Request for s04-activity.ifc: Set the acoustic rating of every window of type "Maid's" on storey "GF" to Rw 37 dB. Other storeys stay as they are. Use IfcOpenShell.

First a look at what the model holds.

```python
import ifcopenshell
import ifcopenshell.util.element

model = ifcopenshell.open("s04-activity.ifc")
print(model.schema)
storey = next(s for s in model.by_type("IfcBuildingStorey") if s.Name == "GF")
windows = [e for e in ifcopenshell.util.element.get_decomposition(storey) if e.is_a("IfcWindow")]
seen = {}
for e in windows:
    element_type = ifcopenshell.util.element.get_type(e)
    key = (element_type.Name if element_type != e and element_type else None, ifcopenshell.util.element.get_pset(e, "Pset_WindowCommon", "AcousticRating"))
    seen[key] = seen.get(key, 0) + 1
for (name, value), count in sorted(seen.items(), key=str):
    print(count, "x", name, "|", value)
```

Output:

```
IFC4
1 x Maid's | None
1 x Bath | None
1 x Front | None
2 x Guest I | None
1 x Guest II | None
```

```python
import ifcopenshell
import ifcopenshell.api.pset
import ifcopenshell.util.element

model = ifcopenshell.open("s04-activity.ifc")

storey = next(s for s in model.by_type("IfcBuildingStorey") if s.Name == "GF")
windows = [e for e in ifcopenshell.util.element.get_decomposition(storey) if e.is_a("IfcWindow")]

count = 0
for e in windows:
    element_type = ifcopenshell.util.element.get_type(e)
    if element_type in (None, e) or element_type.Name != "Maid's":
        continue
    # add_pset returns the element's existing set when there is one.
    pset = ifcopenshell.api.pset.add_pset(model, product=e, name="Pset_WindowCommon")
    ifcopenshell.api.pset.edit_pset(model, pset=pset, properties={"AcousticRating": "Rw 37 dB"})
    count += 1

print(count, "windows updated")

model.write("s04-activity_updated.ifc")
```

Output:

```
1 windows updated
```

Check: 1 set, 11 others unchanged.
